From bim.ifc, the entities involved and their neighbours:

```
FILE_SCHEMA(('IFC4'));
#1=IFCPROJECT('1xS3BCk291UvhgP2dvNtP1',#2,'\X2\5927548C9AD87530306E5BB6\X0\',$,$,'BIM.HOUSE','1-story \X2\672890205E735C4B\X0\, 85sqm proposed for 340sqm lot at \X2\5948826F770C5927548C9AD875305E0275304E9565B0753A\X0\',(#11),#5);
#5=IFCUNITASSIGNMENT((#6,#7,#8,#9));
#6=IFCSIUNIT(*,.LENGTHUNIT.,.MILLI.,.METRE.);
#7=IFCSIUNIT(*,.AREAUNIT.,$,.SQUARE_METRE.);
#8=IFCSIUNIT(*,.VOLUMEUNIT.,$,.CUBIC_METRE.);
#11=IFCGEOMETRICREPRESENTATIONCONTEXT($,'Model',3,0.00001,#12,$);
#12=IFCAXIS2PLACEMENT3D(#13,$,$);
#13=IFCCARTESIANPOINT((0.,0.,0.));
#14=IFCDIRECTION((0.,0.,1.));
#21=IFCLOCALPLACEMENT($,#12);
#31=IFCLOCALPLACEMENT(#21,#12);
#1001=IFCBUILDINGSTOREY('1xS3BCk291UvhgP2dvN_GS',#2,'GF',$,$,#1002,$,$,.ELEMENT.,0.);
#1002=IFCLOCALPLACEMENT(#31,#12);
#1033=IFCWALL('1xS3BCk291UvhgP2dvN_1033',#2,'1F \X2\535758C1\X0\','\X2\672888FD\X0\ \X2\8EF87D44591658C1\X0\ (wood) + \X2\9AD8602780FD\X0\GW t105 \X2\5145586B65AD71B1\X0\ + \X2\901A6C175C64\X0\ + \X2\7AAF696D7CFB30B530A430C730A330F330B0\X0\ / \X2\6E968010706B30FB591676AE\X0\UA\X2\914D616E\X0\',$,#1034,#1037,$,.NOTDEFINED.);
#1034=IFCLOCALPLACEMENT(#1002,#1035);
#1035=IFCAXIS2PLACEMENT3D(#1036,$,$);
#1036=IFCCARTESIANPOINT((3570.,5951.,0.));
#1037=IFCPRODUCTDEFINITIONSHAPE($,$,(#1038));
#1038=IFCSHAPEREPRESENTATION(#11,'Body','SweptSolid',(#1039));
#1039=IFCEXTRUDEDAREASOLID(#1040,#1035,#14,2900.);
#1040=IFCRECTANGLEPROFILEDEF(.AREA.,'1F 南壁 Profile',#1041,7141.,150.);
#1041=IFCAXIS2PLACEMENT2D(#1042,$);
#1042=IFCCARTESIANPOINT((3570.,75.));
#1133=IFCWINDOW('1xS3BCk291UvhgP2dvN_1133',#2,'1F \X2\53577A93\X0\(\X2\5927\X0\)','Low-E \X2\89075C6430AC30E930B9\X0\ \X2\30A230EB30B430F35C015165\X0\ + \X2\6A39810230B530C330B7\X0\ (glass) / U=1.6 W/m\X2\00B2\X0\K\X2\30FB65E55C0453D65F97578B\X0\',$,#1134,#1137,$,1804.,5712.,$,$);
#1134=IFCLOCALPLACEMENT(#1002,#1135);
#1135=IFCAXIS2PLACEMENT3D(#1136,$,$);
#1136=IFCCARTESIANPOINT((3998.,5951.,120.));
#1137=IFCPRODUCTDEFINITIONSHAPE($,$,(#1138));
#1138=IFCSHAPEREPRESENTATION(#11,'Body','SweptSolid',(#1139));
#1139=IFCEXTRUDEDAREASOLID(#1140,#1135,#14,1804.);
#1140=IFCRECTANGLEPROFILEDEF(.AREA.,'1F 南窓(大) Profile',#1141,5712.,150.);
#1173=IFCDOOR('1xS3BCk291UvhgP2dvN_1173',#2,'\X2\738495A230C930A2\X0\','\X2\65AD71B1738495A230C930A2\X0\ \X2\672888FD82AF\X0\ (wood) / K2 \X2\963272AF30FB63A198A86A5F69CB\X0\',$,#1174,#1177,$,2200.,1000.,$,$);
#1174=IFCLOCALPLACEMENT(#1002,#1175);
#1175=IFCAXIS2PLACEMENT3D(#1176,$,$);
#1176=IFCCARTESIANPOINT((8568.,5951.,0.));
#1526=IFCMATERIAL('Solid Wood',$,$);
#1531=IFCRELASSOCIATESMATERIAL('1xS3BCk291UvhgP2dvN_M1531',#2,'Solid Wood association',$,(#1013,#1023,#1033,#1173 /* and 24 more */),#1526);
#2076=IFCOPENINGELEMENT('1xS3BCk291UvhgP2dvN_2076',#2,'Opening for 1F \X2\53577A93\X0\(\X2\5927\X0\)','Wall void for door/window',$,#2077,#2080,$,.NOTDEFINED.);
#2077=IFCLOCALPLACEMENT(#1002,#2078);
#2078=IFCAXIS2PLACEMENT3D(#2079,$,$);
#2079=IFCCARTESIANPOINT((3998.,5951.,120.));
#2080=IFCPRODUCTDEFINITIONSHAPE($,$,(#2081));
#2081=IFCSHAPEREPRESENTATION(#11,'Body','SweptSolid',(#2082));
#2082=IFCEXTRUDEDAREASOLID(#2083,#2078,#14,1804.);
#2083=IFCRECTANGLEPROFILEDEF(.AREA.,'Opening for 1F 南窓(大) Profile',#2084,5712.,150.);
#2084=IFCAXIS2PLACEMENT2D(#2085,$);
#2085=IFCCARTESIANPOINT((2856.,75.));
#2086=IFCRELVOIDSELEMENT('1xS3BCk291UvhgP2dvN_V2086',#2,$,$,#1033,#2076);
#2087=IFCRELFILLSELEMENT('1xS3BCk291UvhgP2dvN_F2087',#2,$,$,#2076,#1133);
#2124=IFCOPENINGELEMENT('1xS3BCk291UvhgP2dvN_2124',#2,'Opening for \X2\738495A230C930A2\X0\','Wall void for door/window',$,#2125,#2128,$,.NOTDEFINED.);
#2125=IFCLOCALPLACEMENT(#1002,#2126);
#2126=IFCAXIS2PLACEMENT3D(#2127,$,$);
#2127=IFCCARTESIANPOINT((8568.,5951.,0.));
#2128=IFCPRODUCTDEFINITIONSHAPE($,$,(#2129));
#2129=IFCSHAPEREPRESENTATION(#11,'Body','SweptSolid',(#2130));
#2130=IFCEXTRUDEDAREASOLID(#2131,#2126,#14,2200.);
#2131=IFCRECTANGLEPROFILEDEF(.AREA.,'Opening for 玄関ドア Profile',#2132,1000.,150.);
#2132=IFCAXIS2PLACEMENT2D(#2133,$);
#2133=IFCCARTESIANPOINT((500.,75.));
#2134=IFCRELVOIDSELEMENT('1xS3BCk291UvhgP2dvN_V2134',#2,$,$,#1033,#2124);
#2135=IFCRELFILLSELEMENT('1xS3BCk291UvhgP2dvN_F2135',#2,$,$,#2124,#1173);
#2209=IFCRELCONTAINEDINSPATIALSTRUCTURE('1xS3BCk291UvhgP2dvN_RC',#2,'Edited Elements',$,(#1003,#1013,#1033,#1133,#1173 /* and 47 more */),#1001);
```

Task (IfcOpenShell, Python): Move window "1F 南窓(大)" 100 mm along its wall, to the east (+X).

```python
import ifcopenshell
import ifcopenshell.api.geometry
import ifcopenshell.util.placement

model = ifcopenshell.open("bim.ifc")

window = model.by_guid("1xS3BCk291UvhgP2dvN_1133")
opening = window.FillsVoids[0].RelatingOpeningElement
wall = opening.VoidsElements[0].RelatingBuildingElement

wall_matrix = ifcopenshell.util.placement.get_local_placement(wall.ObjectPlacement)
shift = wall_matrix[:3, 0] * 100.0
before = ifcopenshell.util.placement.get_local_placement(window.ObjectPlacement)[:3, 3].copy()

# The window is not placed relative to its opening, so move both.
for product in (opening, window):
    matrix = ifcopenshell.util.placement.get_local_placement(product.ObjectPlacement)
    matrix[:3, 3] += shift
    ifcopenshell.api.geometry.edit_object_placement(model, product=product, matrix=matrix, is_si=False)

after = ifcopenshell.util.placement.get_local_placement(window.ObjectPlacement)[:3, 3]
print("window moved by", (after - before).round(3) + 0.0)

model.write("bim_edited.ifc")
```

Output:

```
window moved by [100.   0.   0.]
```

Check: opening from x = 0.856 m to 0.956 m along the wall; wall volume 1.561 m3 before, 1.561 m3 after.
